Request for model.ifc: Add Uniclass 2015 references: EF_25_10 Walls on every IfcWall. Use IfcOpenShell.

First a look at what the model holds.

```python
import ifcopenshell

model = ifcopenshell.open("model.ifc")
print(model.schema)
print("classifications:", [c.Name for c in model.by_type("IfcClassification")])
for ifc_class in ("IfcDoor", "IfcRoof", "IfcStair", "IfcWall", "IfcWindow"):
    print(ifc_class, len(model.by_type(ifc_class)))
```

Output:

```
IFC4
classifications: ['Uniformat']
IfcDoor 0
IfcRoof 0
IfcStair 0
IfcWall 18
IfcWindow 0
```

```python
import ifcopenshell
import ifcopenshell.api.classification

model = ifcopenshell.open("model.ifc")

system = ifcopenshell.api.classification.add_classification(model, classification="Uniclass 2015")

codes = {
    "IfcWall": ("EF_25_10", "Walls"),
}
for ifc_class, (code, name) in codes.items():
    products = model.by_type(ifc_class)
    ifcopenshell.api.classification.add_reference(
        model, products=products, classification=system, identification=code, name=name
    )
    print(code, len(products))

model.write("model_v2.ifc")
```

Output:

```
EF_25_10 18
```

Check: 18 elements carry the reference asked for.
